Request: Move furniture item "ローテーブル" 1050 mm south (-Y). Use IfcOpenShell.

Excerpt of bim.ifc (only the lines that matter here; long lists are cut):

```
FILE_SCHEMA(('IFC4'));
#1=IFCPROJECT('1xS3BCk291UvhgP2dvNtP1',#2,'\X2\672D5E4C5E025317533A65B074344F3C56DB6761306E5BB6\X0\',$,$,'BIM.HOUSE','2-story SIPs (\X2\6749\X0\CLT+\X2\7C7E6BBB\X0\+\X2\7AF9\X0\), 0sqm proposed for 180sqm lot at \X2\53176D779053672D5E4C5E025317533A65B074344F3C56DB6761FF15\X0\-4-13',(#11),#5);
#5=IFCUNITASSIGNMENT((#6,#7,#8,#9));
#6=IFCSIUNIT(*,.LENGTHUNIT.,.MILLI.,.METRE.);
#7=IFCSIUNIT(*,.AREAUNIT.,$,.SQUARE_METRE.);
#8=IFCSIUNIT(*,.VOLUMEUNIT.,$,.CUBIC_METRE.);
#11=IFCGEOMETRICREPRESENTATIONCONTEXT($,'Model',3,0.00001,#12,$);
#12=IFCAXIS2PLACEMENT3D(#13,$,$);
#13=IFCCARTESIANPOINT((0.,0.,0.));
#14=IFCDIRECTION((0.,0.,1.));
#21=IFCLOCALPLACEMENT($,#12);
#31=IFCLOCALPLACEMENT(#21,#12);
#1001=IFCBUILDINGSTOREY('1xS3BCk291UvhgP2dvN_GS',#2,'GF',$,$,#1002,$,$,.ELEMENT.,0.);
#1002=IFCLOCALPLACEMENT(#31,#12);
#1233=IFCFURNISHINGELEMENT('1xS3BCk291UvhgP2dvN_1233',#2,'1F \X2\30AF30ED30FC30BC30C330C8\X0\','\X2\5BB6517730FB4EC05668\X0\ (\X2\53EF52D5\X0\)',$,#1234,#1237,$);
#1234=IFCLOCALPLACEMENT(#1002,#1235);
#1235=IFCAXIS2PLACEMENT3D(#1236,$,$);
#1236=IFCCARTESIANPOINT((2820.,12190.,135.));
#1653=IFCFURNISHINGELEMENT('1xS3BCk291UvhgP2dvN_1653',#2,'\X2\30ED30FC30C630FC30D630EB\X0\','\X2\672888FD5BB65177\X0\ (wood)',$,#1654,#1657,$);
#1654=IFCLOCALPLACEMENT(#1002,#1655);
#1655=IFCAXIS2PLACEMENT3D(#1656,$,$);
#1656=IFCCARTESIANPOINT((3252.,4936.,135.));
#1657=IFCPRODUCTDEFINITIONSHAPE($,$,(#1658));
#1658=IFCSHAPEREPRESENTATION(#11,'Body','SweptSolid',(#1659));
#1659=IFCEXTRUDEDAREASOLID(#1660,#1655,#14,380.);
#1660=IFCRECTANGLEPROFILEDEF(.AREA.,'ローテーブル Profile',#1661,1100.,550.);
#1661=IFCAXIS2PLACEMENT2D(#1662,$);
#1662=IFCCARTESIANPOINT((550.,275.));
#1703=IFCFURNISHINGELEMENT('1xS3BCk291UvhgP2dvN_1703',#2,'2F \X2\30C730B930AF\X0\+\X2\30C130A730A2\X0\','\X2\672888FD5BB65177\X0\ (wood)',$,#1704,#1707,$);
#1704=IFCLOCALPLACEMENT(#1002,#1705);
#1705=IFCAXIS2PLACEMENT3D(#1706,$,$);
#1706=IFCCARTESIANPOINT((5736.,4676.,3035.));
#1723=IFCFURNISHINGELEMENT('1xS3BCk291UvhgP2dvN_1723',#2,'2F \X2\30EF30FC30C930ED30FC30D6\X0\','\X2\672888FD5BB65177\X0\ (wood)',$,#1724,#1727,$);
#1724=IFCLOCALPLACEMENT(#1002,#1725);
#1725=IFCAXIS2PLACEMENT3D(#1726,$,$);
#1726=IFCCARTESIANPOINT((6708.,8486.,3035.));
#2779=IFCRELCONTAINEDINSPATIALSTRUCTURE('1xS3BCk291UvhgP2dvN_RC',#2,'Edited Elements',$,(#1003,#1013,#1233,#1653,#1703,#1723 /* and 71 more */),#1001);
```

```python
import ifcopenshell
import ifcopenshell.api.geometry
import ifcopenshell.util.placement

model = ifcopenshell.open("bim.ifc")

item = model.by_guid("1xS3BCk291UvhgP2dvN_1653")
matrix = ifcopenshell.util.placement.get_local_placement(item.ObjectPlacement)
matrix[1, 3] -= 1050.0
ifcopenshell.api.geometry.edit_object_placement(model, product=item, matrix=matrix, is_si=False)

print(ifcopenshell.util.placement.get_local_placement(item.ObjectPlacement).round(3) + 0.0)

model.write("bim_v2.ifc")
```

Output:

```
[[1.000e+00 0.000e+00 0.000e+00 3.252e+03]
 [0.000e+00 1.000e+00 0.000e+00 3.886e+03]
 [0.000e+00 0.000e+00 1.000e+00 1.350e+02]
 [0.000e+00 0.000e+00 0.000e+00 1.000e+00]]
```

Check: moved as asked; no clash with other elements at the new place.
